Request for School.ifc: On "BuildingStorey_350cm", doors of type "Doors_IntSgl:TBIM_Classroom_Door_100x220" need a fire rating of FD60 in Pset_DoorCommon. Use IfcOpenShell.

First a look at what the model holds.

```python
import ifcopenshell
import ifcopenshell.util.element

model = ifcopenshell.open("School.ifc")
print(model.schema)
storey = next(s for s in model.by_type("IfcBuildingStorey") if s.Name == "BuildingStorey_350cm")
doors = [e for e in ifcopenshell.util.element.get_decomposition(storey) if e.is_a("IfcDoor")]
seen = {}
for e in doors:
    element_type = ifcopenshell.util.element.get_type(e)
    key = (element_type.Name if element_type != e and element_type else None, ifcopenshell.util.element.get_pset(e, "Pset_DoorCommon", "FireRating"))
    seen[key] = seen.get(key, 0) + 1
for (name, value), count in sorted(seen.items(), key=str):
    print(count, "x", name, "|", value)
```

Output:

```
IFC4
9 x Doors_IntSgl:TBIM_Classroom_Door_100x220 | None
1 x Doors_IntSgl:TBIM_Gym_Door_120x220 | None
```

```python
import ifcopenshell
import ifcopenshell.api.pset
import ifcopenshell.util.element

model = ifcopenshell.open("School.ifc")

storey = next(s for s in model.by_type("IfcBuildingStorey") if s.Name == "BuildingStorey_350cm")
doors = [e for e in ifcopenshell.util.element.get_decomposition(storey) if e.is_a("IfcDoor")]

count = 0
for e in doors:
    element_type = ifcopenshell.util.element.get_type(e)
    if element_type in (None, e) or element_type.Name != "Doors_IntSgl:TBIM_Classroom_Door_100x220":
        continue
    # add_pset returns the element's existing set when there is one.
    pset = ifcopenshell.api.pset.add_pset(model, product=e, name="Pset_DoorCommon")
    ifcopenshell.api.pset.edit_pset(model, pset=pset, properties={"FireRating": "FD60"})
    count += 1

print(count, "doors updated")

model.write("School_updated.ifc")
```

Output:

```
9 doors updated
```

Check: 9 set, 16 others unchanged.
